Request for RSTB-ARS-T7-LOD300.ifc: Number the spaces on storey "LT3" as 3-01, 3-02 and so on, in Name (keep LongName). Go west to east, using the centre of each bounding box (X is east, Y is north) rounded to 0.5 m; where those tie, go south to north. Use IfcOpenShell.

First a look at what the model holds.

```python
import ifcopenshell
import ifcopenshell.util.element
import ifcopenshell.util.placement

model = ifcopenshell.open("RSTB-ARS-T7-LOD300.ifc")
print(model.schema)
storey = next(s for s in model.by_type("IfcBuildingStorey") if s.Name == "LT3")
spaces = [e for e in ifcopenshell.util.element.get_decomposition(storey) if e.is_a("IfcSpace")]
for e in sorted(spaces, key=lambda e: e.id()):
    origin = ifcopenshell.util.placement.get_local_placement(e.ObjectPlacement)[:3, 3]
    print(e.id(), e.Name, e.LongName, origin.round(2) + 0.0, sep=" | ")
```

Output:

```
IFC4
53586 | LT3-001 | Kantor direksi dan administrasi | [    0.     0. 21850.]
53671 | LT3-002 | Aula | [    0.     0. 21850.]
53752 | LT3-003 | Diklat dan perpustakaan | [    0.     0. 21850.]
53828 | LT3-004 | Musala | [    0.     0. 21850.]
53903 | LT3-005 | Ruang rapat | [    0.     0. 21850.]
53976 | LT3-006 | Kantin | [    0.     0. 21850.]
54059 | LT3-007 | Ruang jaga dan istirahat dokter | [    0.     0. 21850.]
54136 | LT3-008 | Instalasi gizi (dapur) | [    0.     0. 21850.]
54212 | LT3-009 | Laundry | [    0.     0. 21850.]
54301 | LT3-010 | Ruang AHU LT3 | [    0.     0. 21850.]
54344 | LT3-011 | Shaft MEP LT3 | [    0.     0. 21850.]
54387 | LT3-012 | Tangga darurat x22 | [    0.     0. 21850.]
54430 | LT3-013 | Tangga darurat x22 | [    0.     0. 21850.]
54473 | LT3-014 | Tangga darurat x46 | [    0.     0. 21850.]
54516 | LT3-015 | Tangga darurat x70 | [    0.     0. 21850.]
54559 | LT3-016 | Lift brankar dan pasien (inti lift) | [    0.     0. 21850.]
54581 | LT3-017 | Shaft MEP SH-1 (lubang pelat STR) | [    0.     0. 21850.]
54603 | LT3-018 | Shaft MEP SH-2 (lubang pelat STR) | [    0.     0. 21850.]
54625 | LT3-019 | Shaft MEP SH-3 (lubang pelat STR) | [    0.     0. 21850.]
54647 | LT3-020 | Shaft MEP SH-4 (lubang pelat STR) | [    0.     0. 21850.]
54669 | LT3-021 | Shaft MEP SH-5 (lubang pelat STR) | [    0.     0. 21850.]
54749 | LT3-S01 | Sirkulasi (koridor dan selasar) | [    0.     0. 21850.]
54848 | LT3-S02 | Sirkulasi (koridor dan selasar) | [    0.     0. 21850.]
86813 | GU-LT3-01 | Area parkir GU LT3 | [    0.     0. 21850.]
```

```python
import ifcopenshell
import ifcopenshell.geom
import ifcopenshell.util.element
import ifcopenshell.util.shape

model = ifcopenshell.open("RSTB-ARS-T7-LOD300.ifc")
settings = ifcopenshell.geom.settings()
settings.set("use-world-coords", True)


def centre(element):
    shape = ifcopenshell.geom.create_shape(settings, element)
    return ifcopenshell.util.shape.get_bbox_centroid(shape.geometry)


storey = next(s for s in model.by_type("IfcBuildingStorey") if s.Name == "LT3")
spaces = [e for e in ifcopenshell.util.element.get_decomposition(storey) if e.is_a("IfcSpace")]

# Insertion points can sit at a corner or the storey origin, so sort by the geometry (in metres).
centres = {e: centre(e) for e in spaces}
spaces.sort(key=lambda e: (round(centres[e][0] / 0.5), centres[e][1]))

for i, e in enumerate(spaces, start=1):
    number = f"3-{i:02d}"
    e.Name = number
    print(e.id(), number)

model.write("RSTB-ARS-T7-LOD300_updated.ifc")
```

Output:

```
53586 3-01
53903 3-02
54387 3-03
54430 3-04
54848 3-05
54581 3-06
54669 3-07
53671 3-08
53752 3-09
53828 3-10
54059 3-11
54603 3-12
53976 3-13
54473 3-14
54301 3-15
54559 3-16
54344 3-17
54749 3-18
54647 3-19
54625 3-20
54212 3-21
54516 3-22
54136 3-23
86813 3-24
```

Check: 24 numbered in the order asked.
